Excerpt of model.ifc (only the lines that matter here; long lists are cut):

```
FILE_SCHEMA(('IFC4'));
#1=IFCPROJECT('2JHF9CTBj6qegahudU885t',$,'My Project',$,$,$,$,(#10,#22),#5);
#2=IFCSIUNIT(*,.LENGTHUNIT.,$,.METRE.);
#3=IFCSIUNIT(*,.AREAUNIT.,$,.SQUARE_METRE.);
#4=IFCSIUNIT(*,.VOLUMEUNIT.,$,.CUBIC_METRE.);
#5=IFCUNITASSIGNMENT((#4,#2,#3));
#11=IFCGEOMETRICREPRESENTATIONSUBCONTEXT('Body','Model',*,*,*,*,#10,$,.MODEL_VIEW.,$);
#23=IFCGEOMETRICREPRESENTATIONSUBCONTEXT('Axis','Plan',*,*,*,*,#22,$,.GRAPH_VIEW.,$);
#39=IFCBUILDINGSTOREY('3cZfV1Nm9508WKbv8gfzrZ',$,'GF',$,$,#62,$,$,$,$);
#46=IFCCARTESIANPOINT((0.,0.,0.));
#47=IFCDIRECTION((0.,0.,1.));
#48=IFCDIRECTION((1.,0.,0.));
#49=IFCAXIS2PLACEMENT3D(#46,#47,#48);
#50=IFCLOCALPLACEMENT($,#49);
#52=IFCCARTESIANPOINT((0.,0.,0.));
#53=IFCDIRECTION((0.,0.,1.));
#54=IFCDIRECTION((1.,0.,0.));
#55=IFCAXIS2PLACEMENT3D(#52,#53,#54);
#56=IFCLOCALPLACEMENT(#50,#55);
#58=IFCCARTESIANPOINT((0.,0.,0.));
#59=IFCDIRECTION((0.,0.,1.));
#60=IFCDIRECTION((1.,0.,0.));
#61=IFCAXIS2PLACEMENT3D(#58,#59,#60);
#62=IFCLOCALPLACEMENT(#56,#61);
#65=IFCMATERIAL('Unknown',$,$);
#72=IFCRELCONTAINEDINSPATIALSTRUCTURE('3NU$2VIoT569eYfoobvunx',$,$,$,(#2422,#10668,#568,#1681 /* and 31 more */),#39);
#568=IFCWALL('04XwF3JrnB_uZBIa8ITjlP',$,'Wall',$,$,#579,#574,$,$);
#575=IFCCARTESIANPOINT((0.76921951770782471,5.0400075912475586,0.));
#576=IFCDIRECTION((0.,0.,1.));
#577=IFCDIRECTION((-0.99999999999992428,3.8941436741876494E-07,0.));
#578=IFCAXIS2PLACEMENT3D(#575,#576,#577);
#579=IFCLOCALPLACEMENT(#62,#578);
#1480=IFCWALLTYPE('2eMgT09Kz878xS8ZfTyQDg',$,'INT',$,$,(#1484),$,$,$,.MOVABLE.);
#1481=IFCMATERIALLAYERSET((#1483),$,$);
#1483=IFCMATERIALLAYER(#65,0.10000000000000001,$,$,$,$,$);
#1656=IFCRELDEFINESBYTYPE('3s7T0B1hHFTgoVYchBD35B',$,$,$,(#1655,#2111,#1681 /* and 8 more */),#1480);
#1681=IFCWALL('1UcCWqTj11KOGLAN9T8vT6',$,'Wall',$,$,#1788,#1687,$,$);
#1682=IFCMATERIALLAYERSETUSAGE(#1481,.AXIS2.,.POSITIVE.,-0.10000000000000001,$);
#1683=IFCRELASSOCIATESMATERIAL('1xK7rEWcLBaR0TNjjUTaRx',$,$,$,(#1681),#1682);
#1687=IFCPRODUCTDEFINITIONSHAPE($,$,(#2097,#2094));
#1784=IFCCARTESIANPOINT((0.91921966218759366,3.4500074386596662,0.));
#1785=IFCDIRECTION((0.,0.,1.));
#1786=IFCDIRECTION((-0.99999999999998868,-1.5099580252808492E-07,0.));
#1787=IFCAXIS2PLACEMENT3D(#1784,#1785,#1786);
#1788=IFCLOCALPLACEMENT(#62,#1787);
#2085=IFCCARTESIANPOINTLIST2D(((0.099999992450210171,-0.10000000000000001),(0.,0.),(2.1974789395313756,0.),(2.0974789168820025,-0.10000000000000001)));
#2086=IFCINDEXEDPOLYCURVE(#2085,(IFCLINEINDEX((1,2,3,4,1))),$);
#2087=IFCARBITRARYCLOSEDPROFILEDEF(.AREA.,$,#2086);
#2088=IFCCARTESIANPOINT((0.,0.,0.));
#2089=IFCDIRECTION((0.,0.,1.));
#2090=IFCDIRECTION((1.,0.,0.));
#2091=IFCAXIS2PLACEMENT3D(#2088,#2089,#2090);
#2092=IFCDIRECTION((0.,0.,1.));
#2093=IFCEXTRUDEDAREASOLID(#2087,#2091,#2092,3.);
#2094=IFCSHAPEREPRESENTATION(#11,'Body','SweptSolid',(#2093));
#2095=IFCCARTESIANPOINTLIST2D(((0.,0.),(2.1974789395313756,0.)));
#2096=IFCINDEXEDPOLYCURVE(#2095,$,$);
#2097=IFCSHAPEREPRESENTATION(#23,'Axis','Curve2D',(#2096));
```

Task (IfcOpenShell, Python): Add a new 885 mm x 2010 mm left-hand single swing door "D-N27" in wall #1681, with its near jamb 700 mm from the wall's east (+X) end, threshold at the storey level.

```python
import numpy as np
import ifcopenshell
import ifcopenshell.api.feature
import ifcopenshell.api.geometry
import ifcopenshell.api.root
import ifcopenshell.api.spatial
import ifcopenshell.geom
import ifcopenshell.util.element
import ifcopenshell.util.placement
import ifcopenshell.util.representation
import ifcopenshell.util.shape
import ifcopenshell.util.unit

model = ifcopenshell.open("model.ifc")
unit_scale = ifcopenshell.util.unit.calculate_unit_scale(model)
settings = ifcopenshell.geom.settings()


def volume(element):
    """Net volume in cubic metres, openings subtracted."""
    shape = ifcopenshell.geom.create_shape(settings, element)
    return ifcopenshell.util.shape.get_volume(shape.geometry)


wall = model.by_id(1681)
storey = ifcopenshell.util.element.get_container(wall, ifc_class="IfcBuildingStorey")
context = ifcopenshell.util.representation.get_context(model, "Model", "Body", "MODEL_VIEW")
before = volume(wall)

width, height, from_end, sill = 0.885, 2.01, 0.7, 0.0  # metres

# The wall runs along its own X axis, and the end named is its -X end.
wall_shape = ifcopenshell.geom.create_shape(settings, wall)
x, y, z = ifcopenshell.util.shape.get_vertices(wall_shape.geometry).T
start = x.min() + from_end
face, thickness = float(y.min()), float(y.max() - y.min())
wall_matrix = ifcopenshell.util.placement.get_local_placement(wall.ObjectPlacement)
level = ifcopenshell.util.placement.get_local_placement(storey.ObjectPlacement)[2, 3]


def in_wall(x, y):
    """Placement at x, y metres in the wall's axes, at sill height."""
    matrix = wall_matrix.copy()
    matrix[:, 3] = wall_matrix @ np.array([x / unit_scale, y / unit_scale, 0.0, 1.0])
    matrix[2, 3] = level + sill / unit_scale
    return matrix


# Opening: a box that overshoots both wall faces by 50 mm.
opening = ifcopenshell.api.root.create_entity(model, ifc_class="IfcOpeningElement", predefined_type="OPENING")
box = ifcopenshell.api.geometry.add_wall_representation(
    model, context=context, length=width, height=height, thickness=thickness + 0.1
)
ifcopenshell.api.geometry.assign_representation(model, product=opening, representation=box)
ifcopenshell.api.geometry.edit_object_placement(model, product=opening, matrix=in_wall(start, face - 0.05), is_si=False)
ifcopenshell.api.feature.add_feature(model, feature=opening, element=wall)

door = ifcopenshell.api.root.create_entity(model, ifc_class="IfcDoor", name="D-N27", predefined_type="DOOR")
door.OverallWidth, door.OverallHeight = width / unit_scale, height / unit_scale
door.OperationType = "SINGLE_SWING_LEFT"
body = ifcopenshell.api.geometry.add_door_representation(
    model,
    context=context,
    overall_width=door.OverallWidth,
    overall_height=door.OverallHeight,
    operation_type="SINGLE_SWING_LEFT",
    lining_properties={"LiningDepth": thickness / unit_scale, "ThresholdDepth": thickness / unit_scale},
)
ifcopenshell.api.geometry.assign_representation(model, product=door, representation=body)
ifcopenshell.api.spatial.assign_container(model, products=[door], relating_structure=storey)
ifcopenshell.api.feature.add_filling(model, opening=opening, element=door)

# The lining spans the wall, so the door starts at the wall face.
ifcopenshell.api.geometry.edit_object_placement(model, product=door, matrix=in_wall(start, face), is_si=False)

after = volume(wall)

print(f"wall volume {before:.3f} -> {after:.3f} m3")

model.write("model_edited.ifc")
```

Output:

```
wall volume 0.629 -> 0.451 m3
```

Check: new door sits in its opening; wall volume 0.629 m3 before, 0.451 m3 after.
